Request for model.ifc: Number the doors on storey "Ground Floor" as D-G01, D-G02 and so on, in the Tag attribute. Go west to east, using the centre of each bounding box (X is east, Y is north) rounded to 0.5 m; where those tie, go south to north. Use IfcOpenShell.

First a look at what the model holds.

```python
import ifcopenshell
import ifcopenshell.util.element
import ifcopenshell.util.placement

model = ifcopenshell.open("model.ifc")
print(model.schema)
storey = next(s for s in model.by_type("IfcBuildingStorey") if s.Name == "Ground Floor")
doors = [e for e in ifcopenshell.util.element.get_decomposition(storey) if e.is_a("IfcDoor")]
for e in sorted(doors, key=lambda e: e.id()):
    origin = ifcopenshell.util.placement.get_local_placement(e.ObjectPlacement)[:3, 3]
    print(e.id(), e.Tag, e.Name, origin.round(2) + 0.0, sep=" | ")
```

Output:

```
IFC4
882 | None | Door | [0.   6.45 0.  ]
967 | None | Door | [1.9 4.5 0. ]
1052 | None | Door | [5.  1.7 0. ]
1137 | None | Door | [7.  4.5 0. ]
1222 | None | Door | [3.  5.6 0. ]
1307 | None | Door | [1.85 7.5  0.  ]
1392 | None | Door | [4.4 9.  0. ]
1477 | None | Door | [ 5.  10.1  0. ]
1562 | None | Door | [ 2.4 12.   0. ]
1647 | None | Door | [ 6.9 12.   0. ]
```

```python
import ifcopenshell
import ifcopenshell.geom
import ifcopenshell.util.element
import ifcopenshell.util.shape

model = ifcopenshell.open("model.ifc")
settings = ifcopenshell.geom.settings()
settings.set("use-world-coords", True)


def centre(element):
    shape = ifcopenshell.geom.create_shape(settings, element)
    return ifcopenshell.util.shape.get_bbox_centroid(shape.geometry)


storey = next(s for s in model.by_type("IfcBuildingStorey") if s.Name == "Ground Floor")
doors = [e for e in ifcopenshell.util.element.get_decomposition(storey) if e.is_a("IfcDoor")]

# Insertion points can sit at a corner or the storey origin, so sort by the geometry (in metres).
centres = {e: centre(e) for e in doors}
doors.sort(key=lambda e: (round(centres[e][0] / 0.5), centres[e][1]))

for i, e in enumerate(doors, start=1):
    number = f"D-G{i:02d}"
    e.Tag = number
    print(e.id(), number)

model.write("model_updated.ifc")
```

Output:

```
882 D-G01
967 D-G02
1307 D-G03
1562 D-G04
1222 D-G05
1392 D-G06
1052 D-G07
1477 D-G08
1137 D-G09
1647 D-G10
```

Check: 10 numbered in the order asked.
